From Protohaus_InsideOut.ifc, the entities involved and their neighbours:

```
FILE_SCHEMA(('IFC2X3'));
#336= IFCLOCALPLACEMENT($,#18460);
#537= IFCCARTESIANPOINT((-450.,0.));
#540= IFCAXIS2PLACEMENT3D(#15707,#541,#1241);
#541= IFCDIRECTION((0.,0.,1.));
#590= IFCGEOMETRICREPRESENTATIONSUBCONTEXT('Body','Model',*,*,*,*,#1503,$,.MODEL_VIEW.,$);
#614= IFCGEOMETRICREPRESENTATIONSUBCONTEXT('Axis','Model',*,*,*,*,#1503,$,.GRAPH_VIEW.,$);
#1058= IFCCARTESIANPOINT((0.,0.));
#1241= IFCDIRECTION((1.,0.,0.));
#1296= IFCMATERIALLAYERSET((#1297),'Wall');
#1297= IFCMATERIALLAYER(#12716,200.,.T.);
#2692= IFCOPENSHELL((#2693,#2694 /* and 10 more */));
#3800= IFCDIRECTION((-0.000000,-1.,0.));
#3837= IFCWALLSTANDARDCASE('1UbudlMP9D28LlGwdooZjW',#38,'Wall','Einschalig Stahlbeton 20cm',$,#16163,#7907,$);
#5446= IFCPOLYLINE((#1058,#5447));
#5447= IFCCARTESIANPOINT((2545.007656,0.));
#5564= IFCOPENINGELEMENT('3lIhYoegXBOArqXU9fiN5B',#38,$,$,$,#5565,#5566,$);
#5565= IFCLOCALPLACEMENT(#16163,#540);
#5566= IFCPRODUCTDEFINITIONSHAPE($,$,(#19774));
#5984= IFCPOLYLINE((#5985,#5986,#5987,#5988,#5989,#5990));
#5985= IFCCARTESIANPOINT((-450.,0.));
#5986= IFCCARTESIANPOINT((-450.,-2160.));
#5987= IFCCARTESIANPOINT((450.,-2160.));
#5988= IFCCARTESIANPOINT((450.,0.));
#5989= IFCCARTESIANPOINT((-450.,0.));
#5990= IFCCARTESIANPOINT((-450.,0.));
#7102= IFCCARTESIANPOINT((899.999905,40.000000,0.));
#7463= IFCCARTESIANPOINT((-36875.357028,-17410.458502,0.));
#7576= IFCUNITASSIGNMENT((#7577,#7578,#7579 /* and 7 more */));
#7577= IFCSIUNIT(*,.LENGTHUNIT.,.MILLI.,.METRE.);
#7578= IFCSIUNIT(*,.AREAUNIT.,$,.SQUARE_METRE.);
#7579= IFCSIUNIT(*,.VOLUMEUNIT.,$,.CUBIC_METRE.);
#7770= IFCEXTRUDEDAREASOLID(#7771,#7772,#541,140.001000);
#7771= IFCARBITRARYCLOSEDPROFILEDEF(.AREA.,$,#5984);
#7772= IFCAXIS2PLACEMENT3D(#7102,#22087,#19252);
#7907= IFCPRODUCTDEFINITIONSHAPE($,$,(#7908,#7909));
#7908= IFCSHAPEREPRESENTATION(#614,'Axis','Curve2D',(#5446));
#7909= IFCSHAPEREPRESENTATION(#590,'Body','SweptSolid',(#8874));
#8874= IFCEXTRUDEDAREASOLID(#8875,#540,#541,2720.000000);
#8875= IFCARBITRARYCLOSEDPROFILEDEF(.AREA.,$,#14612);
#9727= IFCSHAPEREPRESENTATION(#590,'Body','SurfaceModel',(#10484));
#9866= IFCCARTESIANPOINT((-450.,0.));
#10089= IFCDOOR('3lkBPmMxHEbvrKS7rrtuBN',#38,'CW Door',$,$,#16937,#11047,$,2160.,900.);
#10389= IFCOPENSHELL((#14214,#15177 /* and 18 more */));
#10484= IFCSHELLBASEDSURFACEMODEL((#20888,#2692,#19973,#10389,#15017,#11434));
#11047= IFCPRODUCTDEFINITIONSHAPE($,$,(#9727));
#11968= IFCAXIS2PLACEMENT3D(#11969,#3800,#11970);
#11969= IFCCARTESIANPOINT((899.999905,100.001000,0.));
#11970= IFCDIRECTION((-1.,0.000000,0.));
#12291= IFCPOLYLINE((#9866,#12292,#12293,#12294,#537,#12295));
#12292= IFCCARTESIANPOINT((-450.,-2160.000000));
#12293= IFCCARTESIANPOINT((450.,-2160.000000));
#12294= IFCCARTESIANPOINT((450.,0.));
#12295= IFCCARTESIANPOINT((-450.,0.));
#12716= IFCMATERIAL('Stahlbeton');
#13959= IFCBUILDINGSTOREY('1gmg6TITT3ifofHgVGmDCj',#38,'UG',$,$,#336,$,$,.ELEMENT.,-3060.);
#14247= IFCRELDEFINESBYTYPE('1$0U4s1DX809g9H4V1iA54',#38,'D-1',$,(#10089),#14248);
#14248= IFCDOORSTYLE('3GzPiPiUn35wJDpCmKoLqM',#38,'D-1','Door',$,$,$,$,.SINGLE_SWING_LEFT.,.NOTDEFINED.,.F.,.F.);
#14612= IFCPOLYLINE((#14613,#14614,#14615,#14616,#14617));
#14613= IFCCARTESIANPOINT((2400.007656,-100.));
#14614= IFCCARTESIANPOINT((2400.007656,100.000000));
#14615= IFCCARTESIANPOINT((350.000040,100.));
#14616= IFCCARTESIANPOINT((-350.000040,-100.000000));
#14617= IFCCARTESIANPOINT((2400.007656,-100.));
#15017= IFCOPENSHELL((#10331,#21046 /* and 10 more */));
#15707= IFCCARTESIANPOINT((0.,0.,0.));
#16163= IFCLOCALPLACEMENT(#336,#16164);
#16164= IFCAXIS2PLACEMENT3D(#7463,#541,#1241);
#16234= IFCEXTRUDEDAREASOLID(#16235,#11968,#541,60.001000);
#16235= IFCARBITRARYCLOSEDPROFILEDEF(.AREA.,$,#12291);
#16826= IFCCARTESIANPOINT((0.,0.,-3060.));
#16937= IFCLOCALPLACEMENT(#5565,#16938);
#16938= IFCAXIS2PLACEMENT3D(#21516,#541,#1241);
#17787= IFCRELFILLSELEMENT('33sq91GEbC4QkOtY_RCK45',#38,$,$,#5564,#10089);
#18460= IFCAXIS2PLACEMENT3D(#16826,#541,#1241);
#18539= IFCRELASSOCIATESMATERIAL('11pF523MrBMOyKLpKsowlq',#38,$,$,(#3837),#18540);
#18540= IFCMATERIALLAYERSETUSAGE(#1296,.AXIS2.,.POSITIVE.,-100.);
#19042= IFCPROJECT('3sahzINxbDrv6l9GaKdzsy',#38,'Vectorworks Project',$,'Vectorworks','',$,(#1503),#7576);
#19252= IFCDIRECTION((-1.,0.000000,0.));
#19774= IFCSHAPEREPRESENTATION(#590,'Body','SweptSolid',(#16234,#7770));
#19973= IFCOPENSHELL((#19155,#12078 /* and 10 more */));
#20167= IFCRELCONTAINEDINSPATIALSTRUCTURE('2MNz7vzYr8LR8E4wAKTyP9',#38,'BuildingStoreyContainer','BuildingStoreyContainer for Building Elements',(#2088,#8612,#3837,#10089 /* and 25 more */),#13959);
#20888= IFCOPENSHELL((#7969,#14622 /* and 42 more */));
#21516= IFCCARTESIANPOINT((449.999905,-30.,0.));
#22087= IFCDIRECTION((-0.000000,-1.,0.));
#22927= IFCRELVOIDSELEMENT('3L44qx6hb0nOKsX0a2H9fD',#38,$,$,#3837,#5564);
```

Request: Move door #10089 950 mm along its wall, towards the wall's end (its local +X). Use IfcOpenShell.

```python
import ifcopenshell
import ifcopenshell.api.geometry
import ifcopenshell.util.placement
import ifcopenshell.util.unit

model = ifcopenshell.open("Protohaus_InsideOut.ifc")
unit_scale = ifcopenshell.util.unit.calculate_unit_scale(model)

door = model.by_id(10089)
opening = door.FillsVoids[0].RelatingOpeningElement
wall = opening.VoidsElements[0].RelatingBuildingElement

wall_matrix = ifcopenshell.util.placement.get_local_placement(wall.ObjectPlacement)
shift = wall_matrix[:3, 0] * 0.95 / unit_scale
before = ifcopenshell.util.placement.get_local_placement(door.ObjectPlacement)[:3, 3].copy()

# The door is placed relative to its opening, so it follows when the opening moves.
matrix = ifcopenshell.util.placement.get_local_placement(opening.ObjectPlacement)
matrix[:3, 3] += shift
ifcopenshell.api.geometry.edit_object_placement(
    model, product=opening, matrix=matrix, is_si=False, should_transform_children=True
)

after = ifcopenshell.util.placement.get_local_placement(door.ObjectPlacement)[:3, 3]
print("door moved by", (after - before).round(3) + 0.0)

model.write("Protohaus_InsideOut_v2.ifc")
```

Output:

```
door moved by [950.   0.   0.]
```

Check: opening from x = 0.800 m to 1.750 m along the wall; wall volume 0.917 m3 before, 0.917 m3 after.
